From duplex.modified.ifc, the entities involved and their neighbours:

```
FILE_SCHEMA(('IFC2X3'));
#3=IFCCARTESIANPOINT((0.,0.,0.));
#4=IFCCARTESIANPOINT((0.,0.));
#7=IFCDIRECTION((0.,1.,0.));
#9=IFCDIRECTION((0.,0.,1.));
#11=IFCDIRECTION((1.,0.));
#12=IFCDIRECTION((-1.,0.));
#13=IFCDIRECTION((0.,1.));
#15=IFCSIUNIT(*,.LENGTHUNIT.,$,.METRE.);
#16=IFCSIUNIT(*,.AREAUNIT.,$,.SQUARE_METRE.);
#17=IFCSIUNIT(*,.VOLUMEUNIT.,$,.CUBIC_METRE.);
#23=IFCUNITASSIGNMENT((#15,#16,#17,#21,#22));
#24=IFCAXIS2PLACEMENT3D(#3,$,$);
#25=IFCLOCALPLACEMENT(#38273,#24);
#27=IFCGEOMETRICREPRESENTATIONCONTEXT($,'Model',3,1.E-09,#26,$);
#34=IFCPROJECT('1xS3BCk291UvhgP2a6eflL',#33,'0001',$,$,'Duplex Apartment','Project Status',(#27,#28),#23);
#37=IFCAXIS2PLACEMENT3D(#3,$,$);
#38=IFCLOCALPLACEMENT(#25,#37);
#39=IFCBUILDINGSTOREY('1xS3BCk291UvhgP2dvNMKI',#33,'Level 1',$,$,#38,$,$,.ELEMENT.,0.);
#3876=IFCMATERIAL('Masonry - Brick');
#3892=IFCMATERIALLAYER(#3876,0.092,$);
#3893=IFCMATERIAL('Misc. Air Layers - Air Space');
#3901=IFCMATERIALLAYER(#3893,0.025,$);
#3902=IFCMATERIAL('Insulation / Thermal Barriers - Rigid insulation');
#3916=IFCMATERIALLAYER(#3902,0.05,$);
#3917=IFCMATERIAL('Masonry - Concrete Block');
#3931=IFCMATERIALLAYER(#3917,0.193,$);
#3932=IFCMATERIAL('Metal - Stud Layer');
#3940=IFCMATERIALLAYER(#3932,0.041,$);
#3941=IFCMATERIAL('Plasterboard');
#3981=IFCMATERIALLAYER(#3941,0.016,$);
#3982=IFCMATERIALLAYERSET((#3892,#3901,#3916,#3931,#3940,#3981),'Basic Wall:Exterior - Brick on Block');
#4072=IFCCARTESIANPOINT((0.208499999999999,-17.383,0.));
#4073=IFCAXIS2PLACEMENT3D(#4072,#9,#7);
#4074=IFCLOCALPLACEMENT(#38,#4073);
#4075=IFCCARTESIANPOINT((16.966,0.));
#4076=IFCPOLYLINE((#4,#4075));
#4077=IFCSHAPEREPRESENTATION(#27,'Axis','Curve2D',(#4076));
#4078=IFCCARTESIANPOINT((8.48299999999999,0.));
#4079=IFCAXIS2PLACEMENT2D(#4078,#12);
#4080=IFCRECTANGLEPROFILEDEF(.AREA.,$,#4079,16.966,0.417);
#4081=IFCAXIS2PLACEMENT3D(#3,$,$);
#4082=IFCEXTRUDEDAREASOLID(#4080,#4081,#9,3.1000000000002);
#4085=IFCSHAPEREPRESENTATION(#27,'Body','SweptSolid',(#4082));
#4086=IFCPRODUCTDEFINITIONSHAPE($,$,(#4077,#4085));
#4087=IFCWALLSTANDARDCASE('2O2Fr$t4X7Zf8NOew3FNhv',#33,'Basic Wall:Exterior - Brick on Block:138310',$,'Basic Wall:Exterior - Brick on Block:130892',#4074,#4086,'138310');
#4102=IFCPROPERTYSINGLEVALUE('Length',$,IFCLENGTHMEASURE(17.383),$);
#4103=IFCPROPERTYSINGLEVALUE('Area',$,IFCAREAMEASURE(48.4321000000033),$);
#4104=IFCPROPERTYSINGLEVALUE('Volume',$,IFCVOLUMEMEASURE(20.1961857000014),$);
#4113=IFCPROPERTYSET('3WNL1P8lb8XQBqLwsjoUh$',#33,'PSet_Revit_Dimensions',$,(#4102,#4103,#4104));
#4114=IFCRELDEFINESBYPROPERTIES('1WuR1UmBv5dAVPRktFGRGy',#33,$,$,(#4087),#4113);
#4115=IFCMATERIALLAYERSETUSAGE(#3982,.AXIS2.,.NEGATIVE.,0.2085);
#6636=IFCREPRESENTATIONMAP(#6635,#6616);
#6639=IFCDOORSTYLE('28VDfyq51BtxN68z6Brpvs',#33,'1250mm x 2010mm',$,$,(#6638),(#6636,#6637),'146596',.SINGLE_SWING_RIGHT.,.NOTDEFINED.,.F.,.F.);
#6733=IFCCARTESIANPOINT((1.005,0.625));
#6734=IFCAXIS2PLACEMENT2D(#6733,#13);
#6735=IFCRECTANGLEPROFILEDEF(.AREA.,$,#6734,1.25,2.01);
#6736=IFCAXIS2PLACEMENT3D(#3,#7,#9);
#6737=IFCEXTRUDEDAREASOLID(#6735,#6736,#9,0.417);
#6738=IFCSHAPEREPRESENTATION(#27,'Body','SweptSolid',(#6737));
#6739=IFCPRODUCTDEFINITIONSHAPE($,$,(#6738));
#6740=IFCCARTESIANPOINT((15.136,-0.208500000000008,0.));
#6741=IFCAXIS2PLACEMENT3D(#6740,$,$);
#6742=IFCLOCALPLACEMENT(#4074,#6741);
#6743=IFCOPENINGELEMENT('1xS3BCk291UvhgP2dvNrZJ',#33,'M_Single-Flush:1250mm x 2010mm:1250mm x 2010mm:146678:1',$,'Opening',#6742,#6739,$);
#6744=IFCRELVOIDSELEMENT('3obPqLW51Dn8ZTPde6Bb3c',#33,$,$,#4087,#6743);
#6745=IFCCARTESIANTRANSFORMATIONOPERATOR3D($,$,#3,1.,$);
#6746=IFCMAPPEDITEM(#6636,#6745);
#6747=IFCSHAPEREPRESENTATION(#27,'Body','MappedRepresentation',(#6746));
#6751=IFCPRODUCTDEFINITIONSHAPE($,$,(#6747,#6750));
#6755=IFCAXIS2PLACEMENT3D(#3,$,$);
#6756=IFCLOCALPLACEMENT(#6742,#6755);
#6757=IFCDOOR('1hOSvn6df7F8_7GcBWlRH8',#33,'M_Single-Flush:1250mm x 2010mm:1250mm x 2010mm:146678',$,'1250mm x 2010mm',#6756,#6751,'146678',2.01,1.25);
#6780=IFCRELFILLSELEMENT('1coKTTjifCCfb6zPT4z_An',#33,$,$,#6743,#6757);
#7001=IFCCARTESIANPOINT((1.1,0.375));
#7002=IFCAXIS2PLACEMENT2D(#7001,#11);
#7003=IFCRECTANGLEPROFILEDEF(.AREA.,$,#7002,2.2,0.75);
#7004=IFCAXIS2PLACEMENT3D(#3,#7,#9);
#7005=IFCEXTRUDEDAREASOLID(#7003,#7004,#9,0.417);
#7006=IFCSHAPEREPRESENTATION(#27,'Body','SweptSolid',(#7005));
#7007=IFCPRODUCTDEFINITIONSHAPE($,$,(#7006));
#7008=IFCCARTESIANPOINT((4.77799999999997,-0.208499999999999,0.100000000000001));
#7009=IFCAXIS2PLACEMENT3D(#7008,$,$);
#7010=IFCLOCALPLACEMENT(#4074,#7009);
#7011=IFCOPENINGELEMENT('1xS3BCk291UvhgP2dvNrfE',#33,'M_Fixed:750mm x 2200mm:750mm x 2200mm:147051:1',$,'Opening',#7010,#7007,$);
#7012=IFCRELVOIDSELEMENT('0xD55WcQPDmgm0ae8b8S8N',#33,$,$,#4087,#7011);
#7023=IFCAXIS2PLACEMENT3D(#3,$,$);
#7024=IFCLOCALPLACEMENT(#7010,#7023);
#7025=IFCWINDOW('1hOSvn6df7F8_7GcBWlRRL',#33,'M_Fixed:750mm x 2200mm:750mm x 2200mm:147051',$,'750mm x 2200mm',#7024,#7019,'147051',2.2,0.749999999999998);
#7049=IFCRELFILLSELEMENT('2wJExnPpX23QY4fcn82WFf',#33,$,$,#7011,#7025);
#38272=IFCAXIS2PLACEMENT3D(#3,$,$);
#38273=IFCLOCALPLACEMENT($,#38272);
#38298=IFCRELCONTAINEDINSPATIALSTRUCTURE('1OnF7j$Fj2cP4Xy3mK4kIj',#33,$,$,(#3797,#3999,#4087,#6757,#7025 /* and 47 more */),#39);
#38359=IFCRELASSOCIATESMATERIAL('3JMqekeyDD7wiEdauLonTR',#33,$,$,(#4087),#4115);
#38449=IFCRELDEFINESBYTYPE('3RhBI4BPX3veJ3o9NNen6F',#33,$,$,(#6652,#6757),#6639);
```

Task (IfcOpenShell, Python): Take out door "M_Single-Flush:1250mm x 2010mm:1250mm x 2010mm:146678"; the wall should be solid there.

```python
import ifcopenshell
import ifcopenshell.api.feature
import ifcopenshell.api.pset
import ifcopenshell.api.root
import ifcopenshell.geom
import ifcopenshell.util.element
import ifcopenshell.util.shape
import ifcopenshell.util.unit

model = ifcopenshell.open("duplex.modified.ifc")
area_scale = ifcopenshell.util.unit.calculate_unit_scale(model, "AREAUNIT")
volume_scale = ifcopenshell.util.unit.calculate_unit_scale(model, "VOLUMEUNIT")
settings = ifcopenshell.geom.settings()


def volume(element):
    """Net volume in cubic metres, openings subtracted."""
    shape = ifcopenshell.geom.create_shape(settings, element)
    return ifcopenshell.util.shape.get_volume(shape.geometry)


door = model.by_id(6757)
opening = door.FillsVoids[0].RelatingOpeningElement
wall = opening.VoidsElements[0].RelatingBuildingElement
before = volume(wall)

ifcopenshell.api.root.remove_product(model, product=door)
ifcopenshell.api.feature.remove_feature(model, feature=opening)

after = volume(wall)
thickness = 0.417  # wall thickness in metres

# Update the wall's stored quantities.
pset = model.by_id(ifcopenshell.util.element.get_pset(wall, "PSet_Revit_Dimensions", should_inherit=False)["id"])
ifcopenshell.api.pset.edit_pset(model, pset=pset, properties={
    "Area": model.create_entity("IfcAreaMeasure", after / thickness / area_scale),
    "Volume": model.create_entity("IfcVolumeMeasure", after / volume_scale),
})

print(f"wall volume {before:.3f} -> {after:.3f} m3")

model.write("duplex.modified_rev.ifc")
```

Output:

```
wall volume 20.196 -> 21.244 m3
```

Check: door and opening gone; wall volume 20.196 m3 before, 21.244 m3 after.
